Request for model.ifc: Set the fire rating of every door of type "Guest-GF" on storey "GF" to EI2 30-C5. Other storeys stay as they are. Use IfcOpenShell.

First a look at what the model holds.

```python
import ifcopenshell
import ifcopenshell.util.element

model = ifcopenshell.open("model.ifc")
print(model.schema)
storey = next(s for s in model.by_type("IfcBuildingStorey") if s.Name == "GF")
doors = [e for e in ifcopenshell.util.element.get_decomposition(storey) if e.is_a("IfcDoor")]
seen = {}
for e in doors:
    element_type = ifcopenshell.util.element.get_type(e)
    key = (element_type.Name if element_type != e and element_type else None, ifcopenshell.util.element.get_pset(e, "Pset_DoorCommon", "FireRating"))
    seen[key] = seen.get(key, 0) + 1
for (name, value), count in sorted(seen.items(), key=str):
    print(count, "x", name, "|", value)
```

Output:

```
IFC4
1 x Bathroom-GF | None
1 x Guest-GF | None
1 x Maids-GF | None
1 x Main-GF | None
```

```python
import ifcopenshell
import ifcopenshell.api.pset
import ifcopenshell.util.element

model = ifcopenshell.open("model.ifc")

storey = next(s for s in model.by_type("IfcBuildingStorey") if s.Name == "GF")
doors = [e for e in ifcopenshell.util.element.get_decomposition(storey) if e.is_a("IfcDoor")]

count = 0
for e in doors:
    element_type = ifcopenshell.util.element.get_type(e)
    if element_type in (None, e) or element_type.Name != "Guest-GF":
        continue
    # add_pset returns the element's existing set when there is one.
    pset = ifcopenshell.api.pset.add_pset(model, product=e, name="Pset_DoorCommon")
    ifcopenshell.api.pset.edit_pset(model, pset=pset, properties={"FireRating": "EI2 30-C5"})
    count += 1

print(count, "doors updated")

model.write("model_v2.ifc")
```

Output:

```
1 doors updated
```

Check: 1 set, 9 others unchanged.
